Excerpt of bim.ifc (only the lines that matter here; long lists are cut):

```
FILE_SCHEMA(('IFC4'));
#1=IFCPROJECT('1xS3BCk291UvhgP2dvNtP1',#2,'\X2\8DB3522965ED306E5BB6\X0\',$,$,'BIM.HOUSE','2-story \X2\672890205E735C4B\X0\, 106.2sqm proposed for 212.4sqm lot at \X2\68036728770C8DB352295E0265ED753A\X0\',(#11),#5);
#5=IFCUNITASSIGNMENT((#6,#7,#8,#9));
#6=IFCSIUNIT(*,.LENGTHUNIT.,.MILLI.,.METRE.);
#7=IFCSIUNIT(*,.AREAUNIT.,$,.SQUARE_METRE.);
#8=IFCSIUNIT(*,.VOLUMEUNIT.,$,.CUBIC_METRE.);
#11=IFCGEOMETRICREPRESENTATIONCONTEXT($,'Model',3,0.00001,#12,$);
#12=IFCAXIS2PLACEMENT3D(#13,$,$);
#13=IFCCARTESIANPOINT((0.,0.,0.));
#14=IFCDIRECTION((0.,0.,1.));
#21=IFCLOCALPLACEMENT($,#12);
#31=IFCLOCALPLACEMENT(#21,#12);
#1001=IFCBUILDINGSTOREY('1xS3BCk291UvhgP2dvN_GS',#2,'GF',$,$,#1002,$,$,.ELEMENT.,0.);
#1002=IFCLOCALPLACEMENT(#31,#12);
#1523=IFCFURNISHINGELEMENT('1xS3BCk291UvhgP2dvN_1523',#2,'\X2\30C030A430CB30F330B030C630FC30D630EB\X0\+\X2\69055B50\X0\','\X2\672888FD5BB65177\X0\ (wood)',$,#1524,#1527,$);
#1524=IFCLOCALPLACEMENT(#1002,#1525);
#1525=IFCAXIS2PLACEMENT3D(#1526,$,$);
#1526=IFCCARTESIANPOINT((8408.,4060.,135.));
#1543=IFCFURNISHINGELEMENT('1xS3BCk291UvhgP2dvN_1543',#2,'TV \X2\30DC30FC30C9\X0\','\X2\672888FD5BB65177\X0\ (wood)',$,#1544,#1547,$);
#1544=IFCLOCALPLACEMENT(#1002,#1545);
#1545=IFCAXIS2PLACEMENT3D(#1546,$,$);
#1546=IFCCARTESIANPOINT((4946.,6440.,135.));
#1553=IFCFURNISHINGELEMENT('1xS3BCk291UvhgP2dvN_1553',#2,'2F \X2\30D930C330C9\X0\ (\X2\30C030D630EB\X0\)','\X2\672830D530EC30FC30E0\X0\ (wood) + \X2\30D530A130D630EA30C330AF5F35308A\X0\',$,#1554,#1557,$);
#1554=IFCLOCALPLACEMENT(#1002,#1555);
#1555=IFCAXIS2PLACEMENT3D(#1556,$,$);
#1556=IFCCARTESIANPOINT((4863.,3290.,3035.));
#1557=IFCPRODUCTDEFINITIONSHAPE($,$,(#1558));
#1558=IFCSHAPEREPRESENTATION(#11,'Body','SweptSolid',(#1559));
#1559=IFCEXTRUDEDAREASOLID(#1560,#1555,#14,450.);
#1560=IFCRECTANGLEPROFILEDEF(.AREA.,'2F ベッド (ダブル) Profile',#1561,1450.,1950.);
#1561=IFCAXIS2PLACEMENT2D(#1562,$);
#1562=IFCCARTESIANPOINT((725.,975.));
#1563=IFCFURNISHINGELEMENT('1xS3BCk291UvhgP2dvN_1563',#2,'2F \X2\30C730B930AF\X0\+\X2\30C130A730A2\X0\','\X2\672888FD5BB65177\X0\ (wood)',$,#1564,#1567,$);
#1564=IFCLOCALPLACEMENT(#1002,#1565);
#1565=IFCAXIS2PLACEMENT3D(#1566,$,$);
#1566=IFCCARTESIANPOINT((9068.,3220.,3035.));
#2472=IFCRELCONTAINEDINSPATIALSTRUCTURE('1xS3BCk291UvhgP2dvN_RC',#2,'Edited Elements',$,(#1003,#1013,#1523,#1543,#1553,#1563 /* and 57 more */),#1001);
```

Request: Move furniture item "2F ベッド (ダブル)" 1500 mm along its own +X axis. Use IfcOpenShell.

```python
import ifcopenshell
import ifcopenshell.api.geometry
import ifcopenshell.util.placement
import ifcopenshell.util.unit

model = ifcopenshell.open("bim.ifc")
unit_scale = ifcopenshell.util.unit.calculate_unit_scale(model)

item = model.by_id(1553)
matrix = ifcopenshell.util.placement.get_local_placement(item.ObjectPlacement)
matrix[:3, 3] += matrix[:3, 0] * 1.5 / unit_scale
ifcopenshell.api.geometry.edit_object_placement(model, product=item, matrix=matrix, is_si=False)

print(ifcopenshell.util.placement.get_local_placement(item.ObjectPlacement).round(3) + 0.0)

model.write("bim_rev.ifc")
```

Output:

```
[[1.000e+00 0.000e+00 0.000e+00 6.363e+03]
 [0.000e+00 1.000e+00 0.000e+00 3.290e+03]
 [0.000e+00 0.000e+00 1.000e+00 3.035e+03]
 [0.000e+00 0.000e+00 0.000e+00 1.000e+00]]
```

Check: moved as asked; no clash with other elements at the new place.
